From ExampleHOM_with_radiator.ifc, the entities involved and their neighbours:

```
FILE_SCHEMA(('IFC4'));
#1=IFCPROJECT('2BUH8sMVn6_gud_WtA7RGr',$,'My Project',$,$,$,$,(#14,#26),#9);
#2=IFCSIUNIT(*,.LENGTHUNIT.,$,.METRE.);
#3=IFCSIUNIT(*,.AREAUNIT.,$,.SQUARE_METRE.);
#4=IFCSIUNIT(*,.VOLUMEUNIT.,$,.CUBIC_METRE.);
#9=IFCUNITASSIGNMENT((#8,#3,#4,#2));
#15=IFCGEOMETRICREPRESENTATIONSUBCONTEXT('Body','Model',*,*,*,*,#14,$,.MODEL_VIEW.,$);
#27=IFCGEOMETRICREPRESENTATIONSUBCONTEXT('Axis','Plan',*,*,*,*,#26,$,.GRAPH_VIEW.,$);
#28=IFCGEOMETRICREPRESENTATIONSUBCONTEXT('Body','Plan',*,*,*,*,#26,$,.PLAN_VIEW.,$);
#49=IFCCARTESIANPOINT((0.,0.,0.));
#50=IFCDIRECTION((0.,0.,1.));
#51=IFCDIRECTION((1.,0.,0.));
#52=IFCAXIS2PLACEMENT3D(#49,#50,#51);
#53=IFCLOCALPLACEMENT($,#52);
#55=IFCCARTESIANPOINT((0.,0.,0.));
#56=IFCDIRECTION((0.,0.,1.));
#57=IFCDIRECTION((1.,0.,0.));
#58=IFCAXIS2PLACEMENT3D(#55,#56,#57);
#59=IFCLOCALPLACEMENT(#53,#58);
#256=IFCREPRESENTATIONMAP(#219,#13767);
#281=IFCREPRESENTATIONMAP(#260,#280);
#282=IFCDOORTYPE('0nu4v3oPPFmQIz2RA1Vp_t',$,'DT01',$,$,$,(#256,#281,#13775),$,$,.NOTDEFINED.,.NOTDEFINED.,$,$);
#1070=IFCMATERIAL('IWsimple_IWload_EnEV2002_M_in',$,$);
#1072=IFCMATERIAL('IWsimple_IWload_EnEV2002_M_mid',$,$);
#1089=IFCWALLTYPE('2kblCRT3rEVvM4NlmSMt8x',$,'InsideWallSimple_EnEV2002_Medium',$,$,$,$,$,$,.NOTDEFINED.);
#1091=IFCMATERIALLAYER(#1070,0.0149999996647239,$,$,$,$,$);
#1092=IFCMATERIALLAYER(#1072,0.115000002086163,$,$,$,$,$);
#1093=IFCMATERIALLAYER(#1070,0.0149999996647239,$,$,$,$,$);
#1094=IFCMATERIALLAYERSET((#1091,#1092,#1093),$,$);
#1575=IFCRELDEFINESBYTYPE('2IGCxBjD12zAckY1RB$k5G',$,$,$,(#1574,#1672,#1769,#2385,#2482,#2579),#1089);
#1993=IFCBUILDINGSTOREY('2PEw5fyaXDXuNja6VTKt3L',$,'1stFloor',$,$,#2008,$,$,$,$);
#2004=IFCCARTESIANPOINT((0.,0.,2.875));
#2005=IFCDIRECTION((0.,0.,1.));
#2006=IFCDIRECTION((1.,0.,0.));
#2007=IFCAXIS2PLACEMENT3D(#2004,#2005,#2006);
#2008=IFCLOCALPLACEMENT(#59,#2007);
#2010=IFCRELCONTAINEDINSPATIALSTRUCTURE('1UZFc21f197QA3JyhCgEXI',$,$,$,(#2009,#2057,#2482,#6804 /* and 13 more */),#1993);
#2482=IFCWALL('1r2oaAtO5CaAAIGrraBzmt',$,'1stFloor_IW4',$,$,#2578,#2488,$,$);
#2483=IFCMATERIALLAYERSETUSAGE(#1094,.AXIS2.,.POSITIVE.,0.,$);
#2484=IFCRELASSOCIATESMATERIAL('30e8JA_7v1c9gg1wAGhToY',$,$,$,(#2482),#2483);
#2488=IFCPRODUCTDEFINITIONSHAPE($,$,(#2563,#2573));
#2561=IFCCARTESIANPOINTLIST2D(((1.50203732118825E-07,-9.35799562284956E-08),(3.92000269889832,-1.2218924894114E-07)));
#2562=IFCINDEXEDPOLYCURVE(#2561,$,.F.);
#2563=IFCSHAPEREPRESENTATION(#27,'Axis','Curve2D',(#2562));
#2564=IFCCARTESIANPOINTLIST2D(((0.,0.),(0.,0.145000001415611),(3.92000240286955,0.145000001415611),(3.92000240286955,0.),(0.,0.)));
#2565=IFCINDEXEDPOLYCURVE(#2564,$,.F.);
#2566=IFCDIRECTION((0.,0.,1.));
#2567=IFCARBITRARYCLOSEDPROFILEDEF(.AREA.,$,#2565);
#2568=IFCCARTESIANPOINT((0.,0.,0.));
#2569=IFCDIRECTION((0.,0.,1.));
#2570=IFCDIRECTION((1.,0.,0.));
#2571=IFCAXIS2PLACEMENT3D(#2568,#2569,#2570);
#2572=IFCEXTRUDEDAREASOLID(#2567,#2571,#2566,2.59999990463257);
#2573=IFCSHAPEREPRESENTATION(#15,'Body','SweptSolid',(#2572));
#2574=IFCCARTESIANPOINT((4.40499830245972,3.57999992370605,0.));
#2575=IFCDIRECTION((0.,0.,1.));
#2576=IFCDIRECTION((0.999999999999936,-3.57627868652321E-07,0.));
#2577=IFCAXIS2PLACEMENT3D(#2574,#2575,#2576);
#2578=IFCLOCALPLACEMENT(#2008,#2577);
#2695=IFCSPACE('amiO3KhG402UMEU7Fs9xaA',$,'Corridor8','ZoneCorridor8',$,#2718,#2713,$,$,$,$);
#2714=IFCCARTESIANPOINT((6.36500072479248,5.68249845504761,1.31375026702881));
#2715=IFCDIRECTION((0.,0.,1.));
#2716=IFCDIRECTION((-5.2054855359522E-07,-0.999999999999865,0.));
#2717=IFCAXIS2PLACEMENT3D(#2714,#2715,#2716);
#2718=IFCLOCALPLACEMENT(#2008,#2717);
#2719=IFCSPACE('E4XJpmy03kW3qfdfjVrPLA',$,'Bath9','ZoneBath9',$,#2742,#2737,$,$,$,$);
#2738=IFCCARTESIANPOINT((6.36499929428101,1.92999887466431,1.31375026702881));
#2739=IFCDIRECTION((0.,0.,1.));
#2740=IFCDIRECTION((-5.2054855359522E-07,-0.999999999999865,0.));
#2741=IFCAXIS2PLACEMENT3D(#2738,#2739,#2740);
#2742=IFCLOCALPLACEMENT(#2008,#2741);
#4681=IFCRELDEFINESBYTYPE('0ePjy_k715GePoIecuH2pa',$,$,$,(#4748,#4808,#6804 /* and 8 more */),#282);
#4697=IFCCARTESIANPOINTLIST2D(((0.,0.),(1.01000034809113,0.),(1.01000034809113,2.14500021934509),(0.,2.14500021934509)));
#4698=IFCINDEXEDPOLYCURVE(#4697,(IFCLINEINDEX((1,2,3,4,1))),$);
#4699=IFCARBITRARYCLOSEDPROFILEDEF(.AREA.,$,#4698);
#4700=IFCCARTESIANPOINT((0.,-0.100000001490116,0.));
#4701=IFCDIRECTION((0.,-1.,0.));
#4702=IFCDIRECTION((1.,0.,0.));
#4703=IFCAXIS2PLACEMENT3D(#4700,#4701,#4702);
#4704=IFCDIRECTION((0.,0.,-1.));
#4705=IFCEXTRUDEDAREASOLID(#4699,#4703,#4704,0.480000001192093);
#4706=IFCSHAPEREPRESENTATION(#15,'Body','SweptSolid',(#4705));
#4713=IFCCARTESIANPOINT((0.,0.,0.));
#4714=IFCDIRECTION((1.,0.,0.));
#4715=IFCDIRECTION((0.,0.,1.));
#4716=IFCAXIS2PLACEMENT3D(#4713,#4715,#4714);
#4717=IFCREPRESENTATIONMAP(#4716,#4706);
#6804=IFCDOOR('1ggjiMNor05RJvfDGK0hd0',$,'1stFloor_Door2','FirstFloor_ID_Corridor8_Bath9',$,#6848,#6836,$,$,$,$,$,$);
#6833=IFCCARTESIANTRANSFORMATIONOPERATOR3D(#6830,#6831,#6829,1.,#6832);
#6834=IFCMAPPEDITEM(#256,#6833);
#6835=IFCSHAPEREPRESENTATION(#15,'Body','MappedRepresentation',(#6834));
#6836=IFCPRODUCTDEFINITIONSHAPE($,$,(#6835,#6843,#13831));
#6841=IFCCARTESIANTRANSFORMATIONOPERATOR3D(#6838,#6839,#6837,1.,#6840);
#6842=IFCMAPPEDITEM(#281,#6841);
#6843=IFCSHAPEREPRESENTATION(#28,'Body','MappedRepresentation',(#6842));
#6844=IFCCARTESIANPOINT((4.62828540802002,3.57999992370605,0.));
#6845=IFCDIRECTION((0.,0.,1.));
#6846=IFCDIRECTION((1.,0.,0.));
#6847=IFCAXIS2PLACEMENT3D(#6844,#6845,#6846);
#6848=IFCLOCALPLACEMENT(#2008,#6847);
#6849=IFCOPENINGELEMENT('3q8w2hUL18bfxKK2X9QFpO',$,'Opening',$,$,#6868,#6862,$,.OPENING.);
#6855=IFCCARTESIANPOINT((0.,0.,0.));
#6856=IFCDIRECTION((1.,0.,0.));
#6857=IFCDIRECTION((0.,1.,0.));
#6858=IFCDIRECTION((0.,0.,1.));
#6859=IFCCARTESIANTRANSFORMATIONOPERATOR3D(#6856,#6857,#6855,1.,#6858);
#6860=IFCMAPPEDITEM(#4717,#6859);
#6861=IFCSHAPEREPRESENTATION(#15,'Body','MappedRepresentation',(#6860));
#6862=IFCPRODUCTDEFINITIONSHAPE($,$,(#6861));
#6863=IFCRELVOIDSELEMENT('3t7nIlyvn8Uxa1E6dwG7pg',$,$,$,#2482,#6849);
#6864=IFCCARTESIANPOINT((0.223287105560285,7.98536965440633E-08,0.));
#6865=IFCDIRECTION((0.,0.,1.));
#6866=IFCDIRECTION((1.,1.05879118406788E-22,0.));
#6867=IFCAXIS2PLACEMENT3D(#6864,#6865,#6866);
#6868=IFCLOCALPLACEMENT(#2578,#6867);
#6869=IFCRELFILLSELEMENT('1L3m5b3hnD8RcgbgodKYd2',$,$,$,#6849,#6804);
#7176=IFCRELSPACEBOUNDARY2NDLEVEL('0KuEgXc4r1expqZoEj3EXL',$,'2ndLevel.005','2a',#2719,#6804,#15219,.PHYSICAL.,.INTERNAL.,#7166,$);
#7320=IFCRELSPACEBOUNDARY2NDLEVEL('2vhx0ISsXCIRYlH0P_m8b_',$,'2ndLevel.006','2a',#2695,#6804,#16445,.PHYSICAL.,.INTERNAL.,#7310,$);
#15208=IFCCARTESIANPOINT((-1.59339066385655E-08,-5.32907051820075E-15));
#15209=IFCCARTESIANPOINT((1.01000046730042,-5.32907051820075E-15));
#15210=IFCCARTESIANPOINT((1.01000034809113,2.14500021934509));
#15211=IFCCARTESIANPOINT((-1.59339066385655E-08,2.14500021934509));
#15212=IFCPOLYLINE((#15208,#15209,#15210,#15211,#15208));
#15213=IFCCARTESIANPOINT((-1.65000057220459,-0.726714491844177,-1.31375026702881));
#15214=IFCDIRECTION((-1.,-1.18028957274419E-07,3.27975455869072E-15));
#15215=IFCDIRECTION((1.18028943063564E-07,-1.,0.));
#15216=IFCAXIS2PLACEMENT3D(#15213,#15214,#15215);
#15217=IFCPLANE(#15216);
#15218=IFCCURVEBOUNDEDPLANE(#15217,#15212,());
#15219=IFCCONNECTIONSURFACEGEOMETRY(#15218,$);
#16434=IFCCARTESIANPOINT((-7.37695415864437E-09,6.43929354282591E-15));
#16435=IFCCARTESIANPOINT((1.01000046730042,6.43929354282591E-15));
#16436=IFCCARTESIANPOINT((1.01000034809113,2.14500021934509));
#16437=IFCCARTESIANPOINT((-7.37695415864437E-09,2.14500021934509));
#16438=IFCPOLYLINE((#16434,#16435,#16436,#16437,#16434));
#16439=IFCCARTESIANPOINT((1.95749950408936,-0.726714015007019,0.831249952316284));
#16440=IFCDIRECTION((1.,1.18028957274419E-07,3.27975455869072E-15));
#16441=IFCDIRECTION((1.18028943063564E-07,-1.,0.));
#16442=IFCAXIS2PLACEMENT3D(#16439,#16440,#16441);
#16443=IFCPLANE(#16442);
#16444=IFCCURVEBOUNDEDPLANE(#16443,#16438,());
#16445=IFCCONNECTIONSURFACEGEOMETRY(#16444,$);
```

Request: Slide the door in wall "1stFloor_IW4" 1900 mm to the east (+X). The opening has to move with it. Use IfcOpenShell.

```python
import numpy as np
import ifcopenshell
import ifcopenshell.api.geometry
import ifcopenshell.util.placement
import ifcopenshell.util.unit

model = ifcopenshell.open("ExampleHOM_with_radiator.ifc")
unit_scale = ifcopenshell.util.unit.calculate_unit_scale(model)

door = model.by_id(6804)
opening = door.FillsVoids[0].RelatingOpeningElement
wall = opening.VoidsElements[0].RelatingBuildingElement

wall_matrix = ifcopenshell.util.placement.get_local_placement(wall.ObjectPlacement)
shift = wall_matrix[:3, 0] * 1.9 / unit_scale
before = ifcopenshell.util.placement.get_local_placement(door.ObjectPlacement)[:3, 3].copy()

# The door is not placed relative to its opening, so move both.
for product in (opening, door):
    matrix = ifcopenshell.util.placement.get_local_placement(product.ObjectPlacement)
    matrix[:3, 3] += shift
    ifcopenshell.api.geometry.edit_object_placement(model, product=product, matrix=matrix, is_si=False)

# Space boundary surfaces are stored in each space's coordinates; move them too.
for rel in door.ProvidesBoundaries:
    if not rel.ConnectionGeometry:
        continue
    surface = rel.ConnectionGeometry.SurfaceOnRelatingElement.BasisSurface
    space_matrix = ifcopenshell.util.placement.get_local_placement(rel.RelatingSpace.ObjectPlacement)
    point = np.array(surface.Position.Location.Coordinates) + space_matrix[:3, :3].T @ shift
    surface.Position = model.createIfcAxis2Placement3D(
        model.createIfcCartesianPoint(point.tolist()), surface.Position.Axis, surface.Position.RefDirection
    )

after = ifcopenshell.util.placement.get_local_placement(door.ObjectPlacement)[:3, 3]
print("door moved by", (after - before).round(3) + 0.0)

model.write("ExampleHOM_with_radiator_edited.ifc")
```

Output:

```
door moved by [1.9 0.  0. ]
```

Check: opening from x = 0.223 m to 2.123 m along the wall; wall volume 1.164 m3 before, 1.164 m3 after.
